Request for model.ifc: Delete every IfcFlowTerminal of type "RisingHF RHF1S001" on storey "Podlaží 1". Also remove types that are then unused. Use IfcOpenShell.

First a look at what the model holds.

```python
import ifcopenshell
import ifcopenshell.util.element

model = ifcopenshell.open("model.ifc")
print(model.schema)
storey = next(s for s in model.by_type("IfcBuildingStorey") if s.Name == "Podlaží 1")
terminals = [e for e in ifcopenshell.util.element.get_decomposition(storey) if e.is_a("IfcFlowTerminal")]
seen = {}
for e in terminals:
    element_type = ifcopenshell.util.element.get_type(e)
    name = element_type.Name if element_type not in (None, e) else None
    seen[name] = seen.get(name, 0) + 1
for name, count in sorted(seen.items(), key=str):
    print(count, "x", name)
```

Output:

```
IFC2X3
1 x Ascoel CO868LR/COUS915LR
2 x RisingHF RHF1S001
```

```python
import ifcopenshell
import ifcopenshell.api.root
import ifcopenshell.util.element

model = ifcopenshell.open("model.ifc")

storey = next(s for s in model.by_type("IfcBuildingStorey") if s.Name == "Podlaží 1")
terminals = [e for e in ifcopenshell.util.element.get_decomposition(storey) if e.is_a("IfcFlowTerminal")]
targets = [e for e in terminals if (t := ifcopenshell.util.element.get_type(e)) not in (None, e) and t.Name == "RisingHF RHF1S001"]
types = {ifcopenshell.util.element.get_type(e) for e in targets} - {None, *targets}

for e in targets:
    ifcopenshell.api.root.remove_product(model, product=e)
print(len(targets), "removed")

unused = [t for t in types if not ifcopenshell.util.element.get_types(t)]
for t in unused:
    ifcopenshell.api.root.remove_product(model, product=t)
print(len(unused), "unused types removed")

model.write("model_rev.ifc")
```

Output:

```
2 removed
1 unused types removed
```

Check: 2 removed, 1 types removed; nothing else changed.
